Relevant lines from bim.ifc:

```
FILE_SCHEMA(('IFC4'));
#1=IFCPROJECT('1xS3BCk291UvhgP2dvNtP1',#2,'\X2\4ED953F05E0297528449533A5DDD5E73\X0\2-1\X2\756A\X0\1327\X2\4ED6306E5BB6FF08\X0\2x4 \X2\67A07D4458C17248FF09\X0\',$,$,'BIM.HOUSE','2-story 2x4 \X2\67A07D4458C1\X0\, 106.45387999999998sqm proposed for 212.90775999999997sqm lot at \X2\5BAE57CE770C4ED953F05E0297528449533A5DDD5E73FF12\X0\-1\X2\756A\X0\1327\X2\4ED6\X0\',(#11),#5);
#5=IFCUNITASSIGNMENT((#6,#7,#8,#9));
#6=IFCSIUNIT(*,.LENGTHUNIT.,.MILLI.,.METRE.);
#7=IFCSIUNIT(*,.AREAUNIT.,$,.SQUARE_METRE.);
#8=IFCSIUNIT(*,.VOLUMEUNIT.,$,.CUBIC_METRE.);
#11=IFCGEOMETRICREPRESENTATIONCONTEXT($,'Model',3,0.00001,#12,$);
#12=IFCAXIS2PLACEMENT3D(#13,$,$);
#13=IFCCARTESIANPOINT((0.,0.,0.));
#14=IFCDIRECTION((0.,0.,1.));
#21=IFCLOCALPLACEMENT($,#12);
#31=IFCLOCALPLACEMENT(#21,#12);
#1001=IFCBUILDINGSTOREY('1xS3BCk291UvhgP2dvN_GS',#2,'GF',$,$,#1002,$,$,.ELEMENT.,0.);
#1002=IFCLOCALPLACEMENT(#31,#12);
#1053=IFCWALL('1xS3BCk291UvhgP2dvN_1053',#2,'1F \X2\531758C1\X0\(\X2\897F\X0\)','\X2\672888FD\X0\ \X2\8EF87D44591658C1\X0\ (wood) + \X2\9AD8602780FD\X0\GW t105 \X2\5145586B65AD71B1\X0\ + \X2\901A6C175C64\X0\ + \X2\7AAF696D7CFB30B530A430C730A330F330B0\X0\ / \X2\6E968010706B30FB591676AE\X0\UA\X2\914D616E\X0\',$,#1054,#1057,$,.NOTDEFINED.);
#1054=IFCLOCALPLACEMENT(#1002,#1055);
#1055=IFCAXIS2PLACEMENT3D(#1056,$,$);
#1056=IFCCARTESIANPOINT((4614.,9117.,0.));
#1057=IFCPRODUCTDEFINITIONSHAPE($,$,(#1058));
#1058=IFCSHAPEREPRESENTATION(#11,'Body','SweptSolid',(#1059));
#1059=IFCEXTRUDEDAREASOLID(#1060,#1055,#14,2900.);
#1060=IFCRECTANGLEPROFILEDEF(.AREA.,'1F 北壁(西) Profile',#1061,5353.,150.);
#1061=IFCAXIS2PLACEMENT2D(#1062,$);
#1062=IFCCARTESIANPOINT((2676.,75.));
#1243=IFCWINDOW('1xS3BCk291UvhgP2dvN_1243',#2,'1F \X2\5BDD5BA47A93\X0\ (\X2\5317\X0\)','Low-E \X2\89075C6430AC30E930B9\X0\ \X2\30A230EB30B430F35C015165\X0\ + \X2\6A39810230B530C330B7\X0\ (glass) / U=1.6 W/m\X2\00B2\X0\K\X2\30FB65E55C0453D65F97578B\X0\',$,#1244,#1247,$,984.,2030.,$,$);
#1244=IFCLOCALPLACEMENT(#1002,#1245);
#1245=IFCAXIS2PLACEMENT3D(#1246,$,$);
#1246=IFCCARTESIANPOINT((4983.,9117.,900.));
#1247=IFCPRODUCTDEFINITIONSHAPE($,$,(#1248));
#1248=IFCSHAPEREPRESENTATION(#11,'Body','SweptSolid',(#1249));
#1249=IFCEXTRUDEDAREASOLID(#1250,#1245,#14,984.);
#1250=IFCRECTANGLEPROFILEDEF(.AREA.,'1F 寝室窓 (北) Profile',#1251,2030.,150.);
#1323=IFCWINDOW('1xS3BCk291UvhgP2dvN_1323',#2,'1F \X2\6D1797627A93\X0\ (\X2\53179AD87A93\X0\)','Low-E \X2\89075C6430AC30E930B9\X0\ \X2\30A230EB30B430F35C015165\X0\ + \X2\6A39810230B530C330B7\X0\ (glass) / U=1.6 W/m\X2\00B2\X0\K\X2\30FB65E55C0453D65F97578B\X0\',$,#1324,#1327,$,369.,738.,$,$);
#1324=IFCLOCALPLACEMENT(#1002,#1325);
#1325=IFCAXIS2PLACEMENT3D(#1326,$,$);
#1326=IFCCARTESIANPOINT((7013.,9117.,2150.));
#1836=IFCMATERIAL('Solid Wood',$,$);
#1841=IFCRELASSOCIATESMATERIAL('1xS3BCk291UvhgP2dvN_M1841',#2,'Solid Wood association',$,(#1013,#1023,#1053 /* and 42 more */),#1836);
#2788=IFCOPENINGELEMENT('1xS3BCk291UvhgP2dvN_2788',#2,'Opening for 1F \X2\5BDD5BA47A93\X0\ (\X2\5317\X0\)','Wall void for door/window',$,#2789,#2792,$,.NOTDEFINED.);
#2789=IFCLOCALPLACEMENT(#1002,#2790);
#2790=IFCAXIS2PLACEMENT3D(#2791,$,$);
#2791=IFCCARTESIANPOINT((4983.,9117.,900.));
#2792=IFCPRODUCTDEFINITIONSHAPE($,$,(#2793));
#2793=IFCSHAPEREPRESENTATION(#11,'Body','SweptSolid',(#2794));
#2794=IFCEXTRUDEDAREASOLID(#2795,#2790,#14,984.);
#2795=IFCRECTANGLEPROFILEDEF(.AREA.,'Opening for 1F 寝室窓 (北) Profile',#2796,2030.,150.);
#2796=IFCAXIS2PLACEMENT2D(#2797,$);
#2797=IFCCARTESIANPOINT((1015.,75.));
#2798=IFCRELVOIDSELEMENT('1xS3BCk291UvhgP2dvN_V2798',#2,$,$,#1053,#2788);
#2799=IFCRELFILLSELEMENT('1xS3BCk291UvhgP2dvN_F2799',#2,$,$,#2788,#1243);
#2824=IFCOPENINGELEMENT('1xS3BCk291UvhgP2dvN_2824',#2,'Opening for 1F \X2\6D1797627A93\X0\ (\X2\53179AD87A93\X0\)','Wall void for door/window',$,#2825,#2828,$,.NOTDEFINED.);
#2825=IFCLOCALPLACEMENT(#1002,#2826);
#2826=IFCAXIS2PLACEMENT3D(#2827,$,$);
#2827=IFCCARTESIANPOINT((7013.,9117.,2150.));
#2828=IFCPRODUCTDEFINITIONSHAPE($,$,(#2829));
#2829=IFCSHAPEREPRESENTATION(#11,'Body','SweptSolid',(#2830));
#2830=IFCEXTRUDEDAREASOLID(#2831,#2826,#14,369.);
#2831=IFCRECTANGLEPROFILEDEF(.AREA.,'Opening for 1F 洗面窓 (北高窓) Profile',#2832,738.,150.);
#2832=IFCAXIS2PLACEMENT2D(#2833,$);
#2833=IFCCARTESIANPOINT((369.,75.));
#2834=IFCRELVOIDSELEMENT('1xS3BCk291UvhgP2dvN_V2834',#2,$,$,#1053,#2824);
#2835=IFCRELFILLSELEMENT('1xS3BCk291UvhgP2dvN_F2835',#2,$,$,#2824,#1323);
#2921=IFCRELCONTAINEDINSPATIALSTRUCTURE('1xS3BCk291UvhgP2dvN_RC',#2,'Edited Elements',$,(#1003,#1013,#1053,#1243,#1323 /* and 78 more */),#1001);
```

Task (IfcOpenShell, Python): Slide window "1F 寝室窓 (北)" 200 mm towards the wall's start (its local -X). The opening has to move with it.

```python
import ifcopenshell
import ifcopenshell.api.geometry
import ifcopenshell.util.placement
import ifcopenshell.util.unit

model = ifcopenshell.open("bim.ifc")
unit_scale = ifcopenshell.util.unit.calculate_unit_scale(model)

window = model.by_id(1243)
opening = window.FillsVoids[0].RelatingOpeningElement
wall = opening.VoidsElements[0].RelatingBuildingElement

wall_matrix = ifcopenshell.util.placement.get_local_placement(wall.ObjectPlacement)
shift = wall_matrix[:3, 0] * -0.2 / unit_scale
before = ifcopenshell.util.placement.get_local_placement(window.ObjectPlacement)[:3, 3].copy()

# The window is not placed relative to its opening, so move both.
for product in (opening, window):
    matrix = ifcopenshell.util.placement.get_local_placement(product.ObjectPlacement)
    matrix[:3, 3] += shift
    ifcopenshell.api.geometry.edit_object_placement(model, product=product, matrix=matrix, is_si=False)

after = ifcopenshell.util.placement.get_local_placement(window.ObjectPlacement)[:3, 3]
print("window moved by", (after - before).round(3) + 0.0)

model.write("bim_edited.ifc")
```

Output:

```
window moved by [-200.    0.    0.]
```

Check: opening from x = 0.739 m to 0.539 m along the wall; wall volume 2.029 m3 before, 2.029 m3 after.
